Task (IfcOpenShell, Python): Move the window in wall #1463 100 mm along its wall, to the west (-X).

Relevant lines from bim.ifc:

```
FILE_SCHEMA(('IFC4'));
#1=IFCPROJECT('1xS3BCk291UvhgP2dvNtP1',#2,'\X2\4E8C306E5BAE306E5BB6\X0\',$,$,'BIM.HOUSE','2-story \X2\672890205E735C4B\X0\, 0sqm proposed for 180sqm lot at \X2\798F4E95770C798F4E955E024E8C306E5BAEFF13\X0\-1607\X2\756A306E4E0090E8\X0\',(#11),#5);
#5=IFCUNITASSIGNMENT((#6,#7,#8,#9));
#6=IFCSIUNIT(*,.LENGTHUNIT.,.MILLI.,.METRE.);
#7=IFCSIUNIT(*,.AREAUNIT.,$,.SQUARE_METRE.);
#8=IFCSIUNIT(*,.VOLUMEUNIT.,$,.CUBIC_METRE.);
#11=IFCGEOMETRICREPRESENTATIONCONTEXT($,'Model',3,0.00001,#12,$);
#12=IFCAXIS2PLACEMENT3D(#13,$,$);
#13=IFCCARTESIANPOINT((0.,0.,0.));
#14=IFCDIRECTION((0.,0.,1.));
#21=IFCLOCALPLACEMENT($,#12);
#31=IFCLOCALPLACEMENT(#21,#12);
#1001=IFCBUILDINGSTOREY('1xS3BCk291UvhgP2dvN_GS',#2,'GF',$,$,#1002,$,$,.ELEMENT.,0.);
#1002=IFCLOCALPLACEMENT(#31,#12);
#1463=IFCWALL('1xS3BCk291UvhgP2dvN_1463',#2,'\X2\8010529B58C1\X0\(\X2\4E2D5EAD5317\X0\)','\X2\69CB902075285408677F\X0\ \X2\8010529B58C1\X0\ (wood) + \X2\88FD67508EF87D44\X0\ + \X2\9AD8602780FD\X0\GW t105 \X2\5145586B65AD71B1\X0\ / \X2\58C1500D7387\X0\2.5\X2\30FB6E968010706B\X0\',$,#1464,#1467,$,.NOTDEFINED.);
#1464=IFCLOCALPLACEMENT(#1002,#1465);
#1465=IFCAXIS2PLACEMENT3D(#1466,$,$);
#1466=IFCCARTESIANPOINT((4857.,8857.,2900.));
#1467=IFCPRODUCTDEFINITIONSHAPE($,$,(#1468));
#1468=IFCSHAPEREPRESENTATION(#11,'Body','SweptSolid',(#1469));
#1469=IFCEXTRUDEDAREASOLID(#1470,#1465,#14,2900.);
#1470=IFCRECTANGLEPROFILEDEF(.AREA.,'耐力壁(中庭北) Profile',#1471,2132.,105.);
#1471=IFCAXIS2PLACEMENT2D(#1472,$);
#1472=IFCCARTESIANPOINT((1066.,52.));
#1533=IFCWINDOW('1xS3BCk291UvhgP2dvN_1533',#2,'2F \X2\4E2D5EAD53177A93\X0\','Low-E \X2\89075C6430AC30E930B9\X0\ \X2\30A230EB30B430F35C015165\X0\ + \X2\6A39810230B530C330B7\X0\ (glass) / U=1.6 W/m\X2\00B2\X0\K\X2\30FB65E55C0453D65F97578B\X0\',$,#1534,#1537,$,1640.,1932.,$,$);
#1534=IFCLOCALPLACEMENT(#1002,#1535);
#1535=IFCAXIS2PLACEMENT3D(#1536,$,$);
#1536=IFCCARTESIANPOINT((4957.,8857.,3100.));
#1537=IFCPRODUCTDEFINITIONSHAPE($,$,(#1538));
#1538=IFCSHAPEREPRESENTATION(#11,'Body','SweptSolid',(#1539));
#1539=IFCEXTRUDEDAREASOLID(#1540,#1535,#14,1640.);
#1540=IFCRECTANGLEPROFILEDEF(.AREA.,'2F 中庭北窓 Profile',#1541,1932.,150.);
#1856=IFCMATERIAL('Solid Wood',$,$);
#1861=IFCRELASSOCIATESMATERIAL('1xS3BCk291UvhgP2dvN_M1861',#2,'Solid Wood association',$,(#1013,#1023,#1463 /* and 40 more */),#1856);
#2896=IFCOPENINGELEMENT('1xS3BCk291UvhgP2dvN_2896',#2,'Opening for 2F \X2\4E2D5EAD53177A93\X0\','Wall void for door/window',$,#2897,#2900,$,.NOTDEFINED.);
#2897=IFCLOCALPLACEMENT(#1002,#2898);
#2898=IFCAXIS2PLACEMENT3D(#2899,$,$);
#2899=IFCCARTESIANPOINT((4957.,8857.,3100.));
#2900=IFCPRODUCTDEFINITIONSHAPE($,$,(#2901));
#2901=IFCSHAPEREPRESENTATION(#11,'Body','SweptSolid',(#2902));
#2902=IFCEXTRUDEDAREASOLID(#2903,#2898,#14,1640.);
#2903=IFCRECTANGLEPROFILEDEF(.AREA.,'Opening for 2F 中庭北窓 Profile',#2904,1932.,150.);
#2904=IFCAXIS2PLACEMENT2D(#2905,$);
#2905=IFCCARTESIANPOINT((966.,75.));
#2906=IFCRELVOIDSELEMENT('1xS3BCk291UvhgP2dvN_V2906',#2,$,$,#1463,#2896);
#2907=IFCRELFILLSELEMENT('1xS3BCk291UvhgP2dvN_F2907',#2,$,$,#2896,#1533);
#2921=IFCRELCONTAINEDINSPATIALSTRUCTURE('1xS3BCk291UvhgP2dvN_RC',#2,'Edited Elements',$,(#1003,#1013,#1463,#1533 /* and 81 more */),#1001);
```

```python
import ifcopenshell
import ifcopenshell.api.geometry
import ifcopenshell.util.placement
import ifcopenshell.util.unit

model = ifcopenshell.open("bim.ifc")
unit_scale = ifcopenshell.util.unit.calculate_unit_scale(model)

window = model.by_id(1533)
opening = window.FillsVoids[0].RelatingOpeningElement
wall = opening.VoidsElements[0].RelatingBuildingElement

wall_matrix = ifcopenshell.util.placement.get_local_placement(wall.ObjectPlacement)
shift = wall_matrix[:3, 0] * -0.1 / unit_scale
before = ifcopenshell.util.placement.get_local_placement(window.ObjectPlacement)[:3, 3].copy()

# The window is not placed relative to its opening, so move both.
for product in (opening, window):
    matrix = ifcopenshell.util.placement.get_local_placement(product.ObjectPlacement)
    matrix[:3, 3] += shift
    ifcopenshell.api.geometry.edit_object_placement(model, product=product, matrix=matrix, is_si=False)

after = ifcopenshell.util.placement.get_local_placement(window.ObjectPlacement)[:3, 3]
print("window moved by", (after - before).round(3) + 0.0)

model.write("bim-out.ifc")
```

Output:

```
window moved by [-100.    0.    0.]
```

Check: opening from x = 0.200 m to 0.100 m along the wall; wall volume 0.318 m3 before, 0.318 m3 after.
